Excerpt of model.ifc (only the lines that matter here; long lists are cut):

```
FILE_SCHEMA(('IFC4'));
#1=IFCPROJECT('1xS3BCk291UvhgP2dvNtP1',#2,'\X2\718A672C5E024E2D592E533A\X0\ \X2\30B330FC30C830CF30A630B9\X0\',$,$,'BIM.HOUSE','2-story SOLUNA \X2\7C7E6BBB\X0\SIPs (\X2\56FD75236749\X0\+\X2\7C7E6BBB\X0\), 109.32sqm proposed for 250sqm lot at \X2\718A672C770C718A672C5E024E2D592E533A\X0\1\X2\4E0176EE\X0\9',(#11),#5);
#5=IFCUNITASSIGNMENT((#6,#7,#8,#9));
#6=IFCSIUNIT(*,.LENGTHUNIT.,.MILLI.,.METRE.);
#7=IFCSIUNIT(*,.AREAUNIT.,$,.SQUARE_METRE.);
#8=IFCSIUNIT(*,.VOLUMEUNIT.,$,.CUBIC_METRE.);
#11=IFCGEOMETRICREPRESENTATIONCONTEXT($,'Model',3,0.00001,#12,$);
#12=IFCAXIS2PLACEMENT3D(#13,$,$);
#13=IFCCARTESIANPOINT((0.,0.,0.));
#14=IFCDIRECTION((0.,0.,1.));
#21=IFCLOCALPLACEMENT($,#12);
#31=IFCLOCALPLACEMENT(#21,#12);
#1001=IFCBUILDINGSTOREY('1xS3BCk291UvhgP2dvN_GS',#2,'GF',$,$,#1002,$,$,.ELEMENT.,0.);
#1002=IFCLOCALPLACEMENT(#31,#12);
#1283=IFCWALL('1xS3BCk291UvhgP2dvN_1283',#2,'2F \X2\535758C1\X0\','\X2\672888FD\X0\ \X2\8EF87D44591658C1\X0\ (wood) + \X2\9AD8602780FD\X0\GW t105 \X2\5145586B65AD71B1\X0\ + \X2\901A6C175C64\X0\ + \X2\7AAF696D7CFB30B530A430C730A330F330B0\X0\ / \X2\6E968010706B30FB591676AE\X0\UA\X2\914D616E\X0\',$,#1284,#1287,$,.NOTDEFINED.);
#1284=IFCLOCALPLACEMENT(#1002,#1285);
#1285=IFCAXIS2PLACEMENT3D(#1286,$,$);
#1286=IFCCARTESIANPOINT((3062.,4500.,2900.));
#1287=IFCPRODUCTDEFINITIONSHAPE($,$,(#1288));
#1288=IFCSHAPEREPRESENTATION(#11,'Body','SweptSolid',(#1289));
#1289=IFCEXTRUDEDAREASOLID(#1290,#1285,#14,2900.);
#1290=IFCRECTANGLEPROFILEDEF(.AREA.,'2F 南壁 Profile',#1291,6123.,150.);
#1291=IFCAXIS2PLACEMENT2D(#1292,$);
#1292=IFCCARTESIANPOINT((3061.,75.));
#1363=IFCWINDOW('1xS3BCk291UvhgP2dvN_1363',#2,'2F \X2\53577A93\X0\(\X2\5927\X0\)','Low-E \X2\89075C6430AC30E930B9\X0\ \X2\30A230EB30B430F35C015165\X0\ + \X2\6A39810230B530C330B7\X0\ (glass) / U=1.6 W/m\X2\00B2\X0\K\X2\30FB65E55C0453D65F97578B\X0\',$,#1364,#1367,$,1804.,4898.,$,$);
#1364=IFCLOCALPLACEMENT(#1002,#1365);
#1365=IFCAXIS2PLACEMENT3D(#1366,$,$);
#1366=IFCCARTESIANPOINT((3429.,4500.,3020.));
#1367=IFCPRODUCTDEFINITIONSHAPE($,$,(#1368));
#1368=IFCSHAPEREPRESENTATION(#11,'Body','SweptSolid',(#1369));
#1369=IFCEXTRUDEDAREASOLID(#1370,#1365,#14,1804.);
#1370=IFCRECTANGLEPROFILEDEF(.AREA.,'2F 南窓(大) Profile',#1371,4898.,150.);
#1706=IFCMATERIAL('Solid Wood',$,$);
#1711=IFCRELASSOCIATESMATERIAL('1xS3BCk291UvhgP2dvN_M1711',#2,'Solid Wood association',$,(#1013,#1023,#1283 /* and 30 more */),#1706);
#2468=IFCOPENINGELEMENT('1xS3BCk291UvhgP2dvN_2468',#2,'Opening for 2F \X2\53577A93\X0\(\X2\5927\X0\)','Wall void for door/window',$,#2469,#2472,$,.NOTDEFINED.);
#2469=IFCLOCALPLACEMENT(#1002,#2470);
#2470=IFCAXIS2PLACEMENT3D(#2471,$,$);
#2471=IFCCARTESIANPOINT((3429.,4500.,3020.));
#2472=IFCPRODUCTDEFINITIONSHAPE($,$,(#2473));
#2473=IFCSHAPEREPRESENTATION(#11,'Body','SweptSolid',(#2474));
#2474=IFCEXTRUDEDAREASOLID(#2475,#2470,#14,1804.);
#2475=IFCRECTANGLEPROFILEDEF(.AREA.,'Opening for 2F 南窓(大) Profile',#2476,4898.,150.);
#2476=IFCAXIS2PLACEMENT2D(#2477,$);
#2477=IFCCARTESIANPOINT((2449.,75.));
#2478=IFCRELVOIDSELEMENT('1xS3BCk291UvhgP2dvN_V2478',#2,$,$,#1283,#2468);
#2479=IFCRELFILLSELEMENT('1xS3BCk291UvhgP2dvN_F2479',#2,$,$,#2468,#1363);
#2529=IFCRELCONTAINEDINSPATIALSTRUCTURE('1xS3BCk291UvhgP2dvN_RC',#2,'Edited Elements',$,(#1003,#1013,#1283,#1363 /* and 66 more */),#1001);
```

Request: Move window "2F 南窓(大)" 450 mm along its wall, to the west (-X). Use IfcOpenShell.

```python
import ifcopenshell
import ifcopenshell.api.geometry
import ifcopenshell.util.placement
import ifcopenshell.util.unit

model = ifcopenshell.open("model.ifc")
unit_scale = ifcopenshell.util.unit.calculate_unit_scale(model)

window = model.by_guid("1xS3BCk291UvhgP2dvN_1363")
opening = window.FillsVoids[0].RelatingOpeningElement
wall = opening.VoidsElements[0].RelatingBuildingElement

wall_matrix = ifcopenshell.util.placement.get_local_placement(wall.ObjectPlacement)
shift = wall_matrix[:3, 0] * -0.45 / unit_scale
before = ifcopenshell.util.placement.get_local_placement(window.ObjectPlacement)[:3, 3].copy()

# The window is not placed relative to its opening, so move both.
for product in (opening, window):
    matrix = ifcopenshell.util.placement.get_local_placement(product.ObjectPlacement)
    matrix[:3, 3] += shift
    ifcopenshell.api.geometry.edit_object_placement(model, product=product, matrix=matrix, is_si=False)

after = ifcopenshell.util.placement.get_local_placement(window.ObjectPlacement)[:3, 3]
print("window moved by", (after - before).round(3) + 0.0)

model.write("model_edited.ifc")
```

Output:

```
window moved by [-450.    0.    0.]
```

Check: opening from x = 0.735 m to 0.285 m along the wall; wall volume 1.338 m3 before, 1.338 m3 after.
